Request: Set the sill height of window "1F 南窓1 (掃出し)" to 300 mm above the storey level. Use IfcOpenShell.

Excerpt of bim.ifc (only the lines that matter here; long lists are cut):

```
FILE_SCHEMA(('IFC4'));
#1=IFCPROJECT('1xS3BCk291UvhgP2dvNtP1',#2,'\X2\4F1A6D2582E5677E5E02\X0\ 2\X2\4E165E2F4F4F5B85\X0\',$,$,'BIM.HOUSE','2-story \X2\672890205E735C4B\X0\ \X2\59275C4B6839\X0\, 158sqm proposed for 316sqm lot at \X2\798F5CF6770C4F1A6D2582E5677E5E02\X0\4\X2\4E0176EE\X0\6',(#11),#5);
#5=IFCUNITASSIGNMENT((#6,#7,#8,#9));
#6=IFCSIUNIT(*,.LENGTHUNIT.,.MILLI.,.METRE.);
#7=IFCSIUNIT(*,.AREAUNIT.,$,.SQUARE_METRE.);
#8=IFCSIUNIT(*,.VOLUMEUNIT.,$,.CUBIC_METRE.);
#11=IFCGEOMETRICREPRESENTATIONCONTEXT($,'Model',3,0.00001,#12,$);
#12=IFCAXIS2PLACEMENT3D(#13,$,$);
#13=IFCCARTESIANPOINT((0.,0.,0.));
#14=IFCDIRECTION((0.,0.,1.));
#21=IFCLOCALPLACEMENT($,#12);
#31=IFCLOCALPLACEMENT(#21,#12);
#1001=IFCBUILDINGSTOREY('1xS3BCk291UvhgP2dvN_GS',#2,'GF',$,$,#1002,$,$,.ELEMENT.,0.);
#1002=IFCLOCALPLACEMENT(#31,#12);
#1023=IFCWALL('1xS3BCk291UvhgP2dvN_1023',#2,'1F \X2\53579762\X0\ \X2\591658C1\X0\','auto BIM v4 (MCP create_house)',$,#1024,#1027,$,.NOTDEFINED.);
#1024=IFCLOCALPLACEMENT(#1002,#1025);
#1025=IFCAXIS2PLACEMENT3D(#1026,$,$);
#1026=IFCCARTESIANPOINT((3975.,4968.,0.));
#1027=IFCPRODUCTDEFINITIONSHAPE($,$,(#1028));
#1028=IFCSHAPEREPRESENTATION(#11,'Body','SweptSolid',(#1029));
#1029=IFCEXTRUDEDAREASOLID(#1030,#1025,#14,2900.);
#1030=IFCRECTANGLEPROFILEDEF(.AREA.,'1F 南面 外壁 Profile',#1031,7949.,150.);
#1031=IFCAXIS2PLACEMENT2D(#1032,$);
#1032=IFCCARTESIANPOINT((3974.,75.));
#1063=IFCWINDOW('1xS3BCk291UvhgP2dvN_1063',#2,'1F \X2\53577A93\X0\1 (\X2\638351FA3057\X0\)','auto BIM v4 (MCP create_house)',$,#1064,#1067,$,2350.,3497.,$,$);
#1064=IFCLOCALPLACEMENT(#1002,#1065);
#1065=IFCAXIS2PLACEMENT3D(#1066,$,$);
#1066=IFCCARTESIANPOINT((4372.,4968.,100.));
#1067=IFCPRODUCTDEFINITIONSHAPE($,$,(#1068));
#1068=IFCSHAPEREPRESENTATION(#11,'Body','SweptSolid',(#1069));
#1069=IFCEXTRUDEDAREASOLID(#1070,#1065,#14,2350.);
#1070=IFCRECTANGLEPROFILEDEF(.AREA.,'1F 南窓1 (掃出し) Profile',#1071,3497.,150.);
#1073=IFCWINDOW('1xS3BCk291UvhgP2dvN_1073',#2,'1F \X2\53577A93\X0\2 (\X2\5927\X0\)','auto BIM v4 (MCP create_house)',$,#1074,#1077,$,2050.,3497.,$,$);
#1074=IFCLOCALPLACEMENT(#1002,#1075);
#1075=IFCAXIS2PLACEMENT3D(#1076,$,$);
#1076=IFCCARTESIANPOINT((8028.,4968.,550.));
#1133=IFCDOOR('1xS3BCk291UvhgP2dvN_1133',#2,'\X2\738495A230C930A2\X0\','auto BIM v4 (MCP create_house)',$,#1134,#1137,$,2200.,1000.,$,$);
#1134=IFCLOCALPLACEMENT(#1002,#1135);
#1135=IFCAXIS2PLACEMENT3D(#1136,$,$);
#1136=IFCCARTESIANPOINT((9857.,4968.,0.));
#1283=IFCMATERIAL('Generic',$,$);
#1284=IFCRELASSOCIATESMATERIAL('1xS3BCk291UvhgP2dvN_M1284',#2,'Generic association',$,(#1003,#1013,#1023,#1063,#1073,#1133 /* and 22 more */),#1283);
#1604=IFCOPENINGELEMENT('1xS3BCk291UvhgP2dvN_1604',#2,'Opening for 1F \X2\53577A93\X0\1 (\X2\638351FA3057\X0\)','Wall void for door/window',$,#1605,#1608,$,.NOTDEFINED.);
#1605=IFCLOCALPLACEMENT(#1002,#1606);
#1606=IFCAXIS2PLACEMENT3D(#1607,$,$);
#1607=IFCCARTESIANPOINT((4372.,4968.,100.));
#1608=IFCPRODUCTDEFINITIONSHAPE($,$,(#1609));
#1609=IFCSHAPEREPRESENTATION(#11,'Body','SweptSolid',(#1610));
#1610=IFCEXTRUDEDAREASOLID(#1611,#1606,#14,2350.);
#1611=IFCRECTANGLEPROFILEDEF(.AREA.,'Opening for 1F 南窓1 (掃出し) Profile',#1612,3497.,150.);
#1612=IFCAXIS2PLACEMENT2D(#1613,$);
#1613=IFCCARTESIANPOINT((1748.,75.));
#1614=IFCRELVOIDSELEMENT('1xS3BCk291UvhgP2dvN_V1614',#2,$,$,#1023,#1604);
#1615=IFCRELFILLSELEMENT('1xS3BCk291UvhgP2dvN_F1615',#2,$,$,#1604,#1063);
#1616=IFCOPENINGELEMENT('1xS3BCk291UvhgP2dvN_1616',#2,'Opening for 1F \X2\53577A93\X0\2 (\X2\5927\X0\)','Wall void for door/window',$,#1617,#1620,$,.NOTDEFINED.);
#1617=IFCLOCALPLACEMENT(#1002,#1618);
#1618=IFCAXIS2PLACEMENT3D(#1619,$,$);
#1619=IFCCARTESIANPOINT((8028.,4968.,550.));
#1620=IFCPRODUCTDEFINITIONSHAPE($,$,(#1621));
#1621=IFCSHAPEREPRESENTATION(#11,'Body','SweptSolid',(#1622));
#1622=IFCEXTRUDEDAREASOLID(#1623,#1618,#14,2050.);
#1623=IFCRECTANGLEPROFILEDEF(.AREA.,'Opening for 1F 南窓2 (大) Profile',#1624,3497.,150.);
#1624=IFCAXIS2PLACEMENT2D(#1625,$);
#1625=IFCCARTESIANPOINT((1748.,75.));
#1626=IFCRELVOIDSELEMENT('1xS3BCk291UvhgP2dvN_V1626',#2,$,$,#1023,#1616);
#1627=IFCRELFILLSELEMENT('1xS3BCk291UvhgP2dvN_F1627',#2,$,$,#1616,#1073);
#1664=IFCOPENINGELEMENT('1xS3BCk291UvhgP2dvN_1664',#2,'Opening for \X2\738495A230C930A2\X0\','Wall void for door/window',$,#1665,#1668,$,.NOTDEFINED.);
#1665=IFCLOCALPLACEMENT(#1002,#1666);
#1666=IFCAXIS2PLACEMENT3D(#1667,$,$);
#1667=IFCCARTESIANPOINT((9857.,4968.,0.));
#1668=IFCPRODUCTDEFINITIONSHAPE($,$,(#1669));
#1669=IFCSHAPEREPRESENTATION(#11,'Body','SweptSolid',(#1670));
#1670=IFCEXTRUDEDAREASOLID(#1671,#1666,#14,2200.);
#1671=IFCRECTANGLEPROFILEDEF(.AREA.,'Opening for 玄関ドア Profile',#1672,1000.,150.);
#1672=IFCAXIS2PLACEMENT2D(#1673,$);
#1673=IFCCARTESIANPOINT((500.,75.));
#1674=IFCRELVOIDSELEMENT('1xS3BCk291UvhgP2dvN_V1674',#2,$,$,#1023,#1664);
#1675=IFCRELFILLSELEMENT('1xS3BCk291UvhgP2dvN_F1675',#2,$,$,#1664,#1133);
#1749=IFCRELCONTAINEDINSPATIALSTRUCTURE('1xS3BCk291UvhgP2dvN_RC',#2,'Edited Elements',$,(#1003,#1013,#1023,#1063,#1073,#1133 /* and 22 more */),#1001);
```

```python
import numpy as np
import ifcopenshell
import ifcopenshell.api.geometry
import ifcopenshell.geom
import ifcopenshell.util.element
import ifcopenshell.util.placement
import ifcopenshell.util.shape
import ifcopenshell.util.unit

model = ifcopenshell.open("bim.ifc")
unit_scale = ifcopenshell.util.unit.calculate_unit_scale(model)

window = model.by_id(1063)
opening = window.FillsVoids[0].RelatingOpeningElement
storey = ifcopenshell.util.element.get_container(window, ifc_class="IfcBuildingStorey")
level = ifcopenshell.util.placement.get_local_placement(storey.ObjectPlacement)[2, 3]

# The opening's origin need not be at the sill, so measure its lowest point.
shape = ifcopenshell.geom.create_shape(ifcopenshell.geom.settings(), opening)
bottom = ifcopenshell.util.shape.get_shape_bottom_elevation(shape, shape.geometry) / unit_scale
dz = level + 0.3 / unit_scale - bottom

shift = np.array([0.0, 0.0, dz])
# The window is not placed relative to its opening, so move both.
for product in (opening, window):
    matrix = ifcopenshell.util.placement.get_local_placement(product.ObjectPlacement)
    matrix[:3, 3] += shift
    ifcopenshell.api.geometry.edit_object_placement(model, product=product, matrix=matrix, is_si=False)

print(f"moved by {dz * unit_scale:+.3f} m")

model.write("bim_updated.ifc")
```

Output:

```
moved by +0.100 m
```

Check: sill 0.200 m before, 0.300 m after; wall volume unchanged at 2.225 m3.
